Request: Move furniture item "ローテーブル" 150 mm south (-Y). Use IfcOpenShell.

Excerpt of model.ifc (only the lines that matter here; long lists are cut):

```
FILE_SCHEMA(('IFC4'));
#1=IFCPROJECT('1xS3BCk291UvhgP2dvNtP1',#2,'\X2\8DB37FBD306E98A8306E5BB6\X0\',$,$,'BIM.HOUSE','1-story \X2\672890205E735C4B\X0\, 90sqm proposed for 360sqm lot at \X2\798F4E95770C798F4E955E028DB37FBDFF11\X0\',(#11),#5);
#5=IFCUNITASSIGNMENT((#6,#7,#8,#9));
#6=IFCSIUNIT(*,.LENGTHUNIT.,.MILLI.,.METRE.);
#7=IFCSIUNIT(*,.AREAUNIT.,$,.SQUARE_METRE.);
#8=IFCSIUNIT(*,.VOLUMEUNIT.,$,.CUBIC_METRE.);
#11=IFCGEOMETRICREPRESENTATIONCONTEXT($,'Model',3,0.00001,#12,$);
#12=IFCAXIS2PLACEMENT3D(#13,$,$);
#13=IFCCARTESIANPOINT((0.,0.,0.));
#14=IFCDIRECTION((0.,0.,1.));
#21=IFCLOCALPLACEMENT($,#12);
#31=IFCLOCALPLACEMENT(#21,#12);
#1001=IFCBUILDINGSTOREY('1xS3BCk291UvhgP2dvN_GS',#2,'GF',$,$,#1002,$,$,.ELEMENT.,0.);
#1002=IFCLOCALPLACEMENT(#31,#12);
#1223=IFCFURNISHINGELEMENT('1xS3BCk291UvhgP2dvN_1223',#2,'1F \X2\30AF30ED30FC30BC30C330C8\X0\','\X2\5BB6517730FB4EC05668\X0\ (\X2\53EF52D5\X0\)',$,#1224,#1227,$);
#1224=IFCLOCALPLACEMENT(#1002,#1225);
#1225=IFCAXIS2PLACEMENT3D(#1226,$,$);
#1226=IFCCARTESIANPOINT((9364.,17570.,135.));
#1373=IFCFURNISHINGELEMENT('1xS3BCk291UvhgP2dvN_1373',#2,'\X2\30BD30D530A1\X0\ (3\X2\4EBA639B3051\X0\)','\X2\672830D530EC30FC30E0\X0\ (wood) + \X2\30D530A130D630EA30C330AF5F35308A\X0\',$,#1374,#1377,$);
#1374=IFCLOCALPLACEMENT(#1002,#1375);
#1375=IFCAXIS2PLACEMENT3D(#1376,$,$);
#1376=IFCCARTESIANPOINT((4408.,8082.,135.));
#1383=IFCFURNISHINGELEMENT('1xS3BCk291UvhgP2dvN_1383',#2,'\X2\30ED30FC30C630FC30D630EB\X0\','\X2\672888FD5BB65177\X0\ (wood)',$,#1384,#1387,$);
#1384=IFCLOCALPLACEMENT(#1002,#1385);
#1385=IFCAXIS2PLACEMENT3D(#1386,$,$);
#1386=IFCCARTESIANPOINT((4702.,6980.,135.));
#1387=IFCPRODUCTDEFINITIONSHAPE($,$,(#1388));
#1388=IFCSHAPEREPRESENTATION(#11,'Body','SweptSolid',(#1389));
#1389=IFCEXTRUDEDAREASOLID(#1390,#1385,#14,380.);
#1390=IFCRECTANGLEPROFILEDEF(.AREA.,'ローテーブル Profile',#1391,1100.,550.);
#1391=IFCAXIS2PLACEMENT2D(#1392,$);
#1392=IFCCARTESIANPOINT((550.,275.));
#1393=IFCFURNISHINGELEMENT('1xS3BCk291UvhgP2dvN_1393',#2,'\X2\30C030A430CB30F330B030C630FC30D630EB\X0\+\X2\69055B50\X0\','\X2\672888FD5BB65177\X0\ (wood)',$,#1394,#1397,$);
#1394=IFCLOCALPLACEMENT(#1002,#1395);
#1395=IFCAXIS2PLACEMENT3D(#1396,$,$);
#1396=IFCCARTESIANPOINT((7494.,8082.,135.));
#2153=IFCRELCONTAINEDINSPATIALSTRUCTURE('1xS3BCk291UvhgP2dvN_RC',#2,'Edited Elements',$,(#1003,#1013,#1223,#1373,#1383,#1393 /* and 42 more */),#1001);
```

```python
import ifcopenshell
import ifcopenshell.api.geometry
import ifcopenshell.util.placement

model = ifcopenshell.open("model.ifc")

item = model.by_guid("1xS3BCk291UvhgP2dvN_1383")
matrix = ifcopenshell.util.placement.get_local_placement(item.ObjectPlacement)
matrix[1, 3] -= 150.0
ifcopenshell.api.geometry.edit_object_placement(model, product=item, matrix=matrix, is_si=False)

print(ifcopenshell.util.placement.get_local_placement(item.ObjectPlacement).round(3) + 0.0)

model.write("model_updated.ifc")
```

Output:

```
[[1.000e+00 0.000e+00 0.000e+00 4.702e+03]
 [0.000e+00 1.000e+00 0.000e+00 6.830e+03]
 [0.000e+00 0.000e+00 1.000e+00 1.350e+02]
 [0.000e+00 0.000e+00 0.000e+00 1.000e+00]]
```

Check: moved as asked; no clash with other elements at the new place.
